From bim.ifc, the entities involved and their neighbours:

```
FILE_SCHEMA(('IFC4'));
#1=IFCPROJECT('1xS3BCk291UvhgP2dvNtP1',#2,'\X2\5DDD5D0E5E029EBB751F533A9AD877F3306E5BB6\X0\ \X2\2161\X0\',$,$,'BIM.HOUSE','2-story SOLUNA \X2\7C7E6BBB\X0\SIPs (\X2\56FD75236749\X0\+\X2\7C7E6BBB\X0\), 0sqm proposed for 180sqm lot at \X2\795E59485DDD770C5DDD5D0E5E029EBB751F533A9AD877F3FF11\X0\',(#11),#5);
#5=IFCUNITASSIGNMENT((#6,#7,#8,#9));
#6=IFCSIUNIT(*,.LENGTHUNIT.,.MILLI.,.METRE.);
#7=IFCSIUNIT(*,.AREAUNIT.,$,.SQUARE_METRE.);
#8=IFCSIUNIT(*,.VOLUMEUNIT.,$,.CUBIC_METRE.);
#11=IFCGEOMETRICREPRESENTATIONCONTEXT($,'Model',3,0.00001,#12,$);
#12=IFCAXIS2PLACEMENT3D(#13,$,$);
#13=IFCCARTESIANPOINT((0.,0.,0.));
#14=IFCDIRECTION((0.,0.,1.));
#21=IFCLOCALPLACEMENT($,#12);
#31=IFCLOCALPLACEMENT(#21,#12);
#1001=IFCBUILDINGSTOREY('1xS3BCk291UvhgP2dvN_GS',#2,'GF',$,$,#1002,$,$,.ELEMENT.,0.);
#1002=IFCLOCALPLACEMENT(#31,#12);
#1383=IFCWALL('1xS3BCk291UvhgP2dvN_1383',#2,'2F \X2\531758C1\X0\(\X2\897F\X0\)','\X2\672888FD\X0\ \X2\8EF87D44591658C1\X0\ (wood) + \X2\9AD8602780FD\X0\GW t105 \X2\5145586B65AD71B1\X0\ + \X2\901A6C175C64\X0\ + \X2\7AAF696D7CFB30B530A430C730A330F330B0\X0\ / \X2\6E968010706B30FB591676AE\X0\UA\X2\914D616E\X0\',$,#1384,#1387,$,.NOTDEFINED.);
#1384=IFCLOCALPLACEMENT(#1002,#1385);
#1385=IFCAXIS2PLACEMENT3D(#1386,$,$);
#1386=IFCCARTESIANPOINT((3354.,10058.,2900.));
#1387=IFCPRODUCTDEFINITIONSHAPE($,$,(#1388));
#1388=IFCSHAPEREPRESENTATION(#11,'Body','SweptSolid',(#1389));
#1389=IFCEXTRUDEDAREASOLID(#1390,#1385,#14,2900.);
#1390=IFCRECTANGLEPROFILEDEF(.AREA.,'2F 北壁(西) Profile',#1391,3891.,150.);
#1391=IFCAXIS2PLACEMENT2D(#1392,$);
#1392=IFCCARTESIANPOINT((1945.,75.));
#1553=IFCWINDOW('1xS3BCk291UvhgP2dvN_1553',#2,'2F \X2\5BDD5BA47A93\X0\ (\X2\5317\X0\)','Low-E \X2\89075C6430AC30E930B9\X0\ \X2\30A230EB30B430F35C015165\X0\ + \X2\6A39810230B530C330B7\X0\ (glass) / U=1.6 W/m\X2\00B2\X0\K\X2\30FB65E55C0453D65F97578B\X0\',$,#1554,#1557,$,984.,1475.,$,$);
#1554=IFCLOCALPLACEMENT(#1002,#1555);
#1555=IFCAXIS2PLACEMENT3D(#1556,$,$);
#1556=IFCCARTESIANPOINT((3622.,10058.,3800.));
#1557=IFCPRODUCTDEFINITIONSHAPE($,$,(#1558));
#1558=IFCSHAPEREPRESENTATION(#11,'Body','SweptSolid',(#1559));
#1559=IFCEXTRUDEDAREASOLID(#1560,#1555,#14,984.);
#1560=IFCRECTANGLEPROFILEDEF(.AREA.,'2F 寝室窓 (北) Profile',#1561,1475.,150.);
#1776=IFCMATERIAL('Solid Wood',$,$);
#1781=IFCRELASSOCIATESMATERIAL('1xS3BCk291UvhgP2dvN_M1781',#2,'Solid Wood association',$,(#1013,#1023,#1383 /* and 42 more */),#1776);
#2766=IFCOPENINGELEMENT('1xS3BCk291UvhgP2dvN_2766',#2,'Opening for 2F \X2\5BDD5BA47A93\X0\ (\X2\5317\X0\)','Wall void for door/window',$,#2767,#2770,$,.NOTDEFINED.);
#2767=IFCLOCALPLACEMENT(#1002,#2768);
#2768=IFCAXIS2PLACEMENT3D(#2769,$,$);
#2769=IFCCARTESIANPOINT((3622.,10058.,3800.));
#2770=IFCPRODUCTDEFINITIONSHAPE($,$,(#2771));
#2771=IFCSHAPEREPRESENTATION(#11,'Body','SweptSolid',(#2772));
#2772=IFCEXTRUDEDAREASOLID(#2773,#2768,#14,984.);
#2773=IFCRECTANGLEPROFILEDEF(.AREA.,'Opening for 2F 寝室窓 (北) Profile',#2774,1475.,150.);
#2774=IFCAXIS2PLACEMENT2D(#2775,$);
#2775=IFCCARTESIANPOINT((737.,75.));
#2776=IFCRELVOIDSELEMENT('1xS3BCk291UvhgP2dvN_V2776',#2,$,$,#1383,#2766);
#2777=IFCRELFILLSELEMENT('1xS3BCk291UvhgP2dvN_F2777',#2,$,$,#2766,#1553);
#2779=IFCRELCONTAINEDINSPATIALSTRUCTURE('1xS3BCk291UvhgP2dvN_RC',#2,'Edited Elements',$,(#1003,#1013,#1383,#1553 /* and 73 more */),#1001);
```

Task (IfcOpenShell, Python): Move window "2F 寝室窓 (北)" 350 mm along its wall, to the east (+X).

```python
import ifcopenshell
import ifcopenshell.api.geometry
import ifcopenshell.util.placement
import ifcopenshell.util.unit

model = ifcopenshell.open("bim.ifc")
unit_scale = ifcopenshell.util.unit.calculate_unit_scale(model)

window = model.by_id(1553)
opening = window.FillsVoids[0].RelatingOpeningElement
wall = opening.VoidsElements[0].RelatingBuildingElement

wall_matrix = ifcopenshell.util.placement.get_local_placement(wall.ObjectPlacement)
shift = wall_matrix[:3, 0] * 0.35 / unit_scale
before = ifcopenshell.util.placement.get_local_placement(window.ObjectPlacement)[:3, 3].copy()

# The window is not placed relative to its opening, so move both.
for product in (opening, window):
    matrix = ifcopenshell.util.placement.get_local_placement(product.ObjectPlacement)
    matrix[:3, 3] += shift
    ifcopenshell.api.geometry.edit_object_placement(model, product=product, matrix=matrix, is_si=False)

after = ifcopenshell.util.placement.get_local_placement(window.ObjectPlacement)[:3, 3]
print("window moved by", (after - before).round(3) + 0.0)

model.write("bim_v2.ifc")
```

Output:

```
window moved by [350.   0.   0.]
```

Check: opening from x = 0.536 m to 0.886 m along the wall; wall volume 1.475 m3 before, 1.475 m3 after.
